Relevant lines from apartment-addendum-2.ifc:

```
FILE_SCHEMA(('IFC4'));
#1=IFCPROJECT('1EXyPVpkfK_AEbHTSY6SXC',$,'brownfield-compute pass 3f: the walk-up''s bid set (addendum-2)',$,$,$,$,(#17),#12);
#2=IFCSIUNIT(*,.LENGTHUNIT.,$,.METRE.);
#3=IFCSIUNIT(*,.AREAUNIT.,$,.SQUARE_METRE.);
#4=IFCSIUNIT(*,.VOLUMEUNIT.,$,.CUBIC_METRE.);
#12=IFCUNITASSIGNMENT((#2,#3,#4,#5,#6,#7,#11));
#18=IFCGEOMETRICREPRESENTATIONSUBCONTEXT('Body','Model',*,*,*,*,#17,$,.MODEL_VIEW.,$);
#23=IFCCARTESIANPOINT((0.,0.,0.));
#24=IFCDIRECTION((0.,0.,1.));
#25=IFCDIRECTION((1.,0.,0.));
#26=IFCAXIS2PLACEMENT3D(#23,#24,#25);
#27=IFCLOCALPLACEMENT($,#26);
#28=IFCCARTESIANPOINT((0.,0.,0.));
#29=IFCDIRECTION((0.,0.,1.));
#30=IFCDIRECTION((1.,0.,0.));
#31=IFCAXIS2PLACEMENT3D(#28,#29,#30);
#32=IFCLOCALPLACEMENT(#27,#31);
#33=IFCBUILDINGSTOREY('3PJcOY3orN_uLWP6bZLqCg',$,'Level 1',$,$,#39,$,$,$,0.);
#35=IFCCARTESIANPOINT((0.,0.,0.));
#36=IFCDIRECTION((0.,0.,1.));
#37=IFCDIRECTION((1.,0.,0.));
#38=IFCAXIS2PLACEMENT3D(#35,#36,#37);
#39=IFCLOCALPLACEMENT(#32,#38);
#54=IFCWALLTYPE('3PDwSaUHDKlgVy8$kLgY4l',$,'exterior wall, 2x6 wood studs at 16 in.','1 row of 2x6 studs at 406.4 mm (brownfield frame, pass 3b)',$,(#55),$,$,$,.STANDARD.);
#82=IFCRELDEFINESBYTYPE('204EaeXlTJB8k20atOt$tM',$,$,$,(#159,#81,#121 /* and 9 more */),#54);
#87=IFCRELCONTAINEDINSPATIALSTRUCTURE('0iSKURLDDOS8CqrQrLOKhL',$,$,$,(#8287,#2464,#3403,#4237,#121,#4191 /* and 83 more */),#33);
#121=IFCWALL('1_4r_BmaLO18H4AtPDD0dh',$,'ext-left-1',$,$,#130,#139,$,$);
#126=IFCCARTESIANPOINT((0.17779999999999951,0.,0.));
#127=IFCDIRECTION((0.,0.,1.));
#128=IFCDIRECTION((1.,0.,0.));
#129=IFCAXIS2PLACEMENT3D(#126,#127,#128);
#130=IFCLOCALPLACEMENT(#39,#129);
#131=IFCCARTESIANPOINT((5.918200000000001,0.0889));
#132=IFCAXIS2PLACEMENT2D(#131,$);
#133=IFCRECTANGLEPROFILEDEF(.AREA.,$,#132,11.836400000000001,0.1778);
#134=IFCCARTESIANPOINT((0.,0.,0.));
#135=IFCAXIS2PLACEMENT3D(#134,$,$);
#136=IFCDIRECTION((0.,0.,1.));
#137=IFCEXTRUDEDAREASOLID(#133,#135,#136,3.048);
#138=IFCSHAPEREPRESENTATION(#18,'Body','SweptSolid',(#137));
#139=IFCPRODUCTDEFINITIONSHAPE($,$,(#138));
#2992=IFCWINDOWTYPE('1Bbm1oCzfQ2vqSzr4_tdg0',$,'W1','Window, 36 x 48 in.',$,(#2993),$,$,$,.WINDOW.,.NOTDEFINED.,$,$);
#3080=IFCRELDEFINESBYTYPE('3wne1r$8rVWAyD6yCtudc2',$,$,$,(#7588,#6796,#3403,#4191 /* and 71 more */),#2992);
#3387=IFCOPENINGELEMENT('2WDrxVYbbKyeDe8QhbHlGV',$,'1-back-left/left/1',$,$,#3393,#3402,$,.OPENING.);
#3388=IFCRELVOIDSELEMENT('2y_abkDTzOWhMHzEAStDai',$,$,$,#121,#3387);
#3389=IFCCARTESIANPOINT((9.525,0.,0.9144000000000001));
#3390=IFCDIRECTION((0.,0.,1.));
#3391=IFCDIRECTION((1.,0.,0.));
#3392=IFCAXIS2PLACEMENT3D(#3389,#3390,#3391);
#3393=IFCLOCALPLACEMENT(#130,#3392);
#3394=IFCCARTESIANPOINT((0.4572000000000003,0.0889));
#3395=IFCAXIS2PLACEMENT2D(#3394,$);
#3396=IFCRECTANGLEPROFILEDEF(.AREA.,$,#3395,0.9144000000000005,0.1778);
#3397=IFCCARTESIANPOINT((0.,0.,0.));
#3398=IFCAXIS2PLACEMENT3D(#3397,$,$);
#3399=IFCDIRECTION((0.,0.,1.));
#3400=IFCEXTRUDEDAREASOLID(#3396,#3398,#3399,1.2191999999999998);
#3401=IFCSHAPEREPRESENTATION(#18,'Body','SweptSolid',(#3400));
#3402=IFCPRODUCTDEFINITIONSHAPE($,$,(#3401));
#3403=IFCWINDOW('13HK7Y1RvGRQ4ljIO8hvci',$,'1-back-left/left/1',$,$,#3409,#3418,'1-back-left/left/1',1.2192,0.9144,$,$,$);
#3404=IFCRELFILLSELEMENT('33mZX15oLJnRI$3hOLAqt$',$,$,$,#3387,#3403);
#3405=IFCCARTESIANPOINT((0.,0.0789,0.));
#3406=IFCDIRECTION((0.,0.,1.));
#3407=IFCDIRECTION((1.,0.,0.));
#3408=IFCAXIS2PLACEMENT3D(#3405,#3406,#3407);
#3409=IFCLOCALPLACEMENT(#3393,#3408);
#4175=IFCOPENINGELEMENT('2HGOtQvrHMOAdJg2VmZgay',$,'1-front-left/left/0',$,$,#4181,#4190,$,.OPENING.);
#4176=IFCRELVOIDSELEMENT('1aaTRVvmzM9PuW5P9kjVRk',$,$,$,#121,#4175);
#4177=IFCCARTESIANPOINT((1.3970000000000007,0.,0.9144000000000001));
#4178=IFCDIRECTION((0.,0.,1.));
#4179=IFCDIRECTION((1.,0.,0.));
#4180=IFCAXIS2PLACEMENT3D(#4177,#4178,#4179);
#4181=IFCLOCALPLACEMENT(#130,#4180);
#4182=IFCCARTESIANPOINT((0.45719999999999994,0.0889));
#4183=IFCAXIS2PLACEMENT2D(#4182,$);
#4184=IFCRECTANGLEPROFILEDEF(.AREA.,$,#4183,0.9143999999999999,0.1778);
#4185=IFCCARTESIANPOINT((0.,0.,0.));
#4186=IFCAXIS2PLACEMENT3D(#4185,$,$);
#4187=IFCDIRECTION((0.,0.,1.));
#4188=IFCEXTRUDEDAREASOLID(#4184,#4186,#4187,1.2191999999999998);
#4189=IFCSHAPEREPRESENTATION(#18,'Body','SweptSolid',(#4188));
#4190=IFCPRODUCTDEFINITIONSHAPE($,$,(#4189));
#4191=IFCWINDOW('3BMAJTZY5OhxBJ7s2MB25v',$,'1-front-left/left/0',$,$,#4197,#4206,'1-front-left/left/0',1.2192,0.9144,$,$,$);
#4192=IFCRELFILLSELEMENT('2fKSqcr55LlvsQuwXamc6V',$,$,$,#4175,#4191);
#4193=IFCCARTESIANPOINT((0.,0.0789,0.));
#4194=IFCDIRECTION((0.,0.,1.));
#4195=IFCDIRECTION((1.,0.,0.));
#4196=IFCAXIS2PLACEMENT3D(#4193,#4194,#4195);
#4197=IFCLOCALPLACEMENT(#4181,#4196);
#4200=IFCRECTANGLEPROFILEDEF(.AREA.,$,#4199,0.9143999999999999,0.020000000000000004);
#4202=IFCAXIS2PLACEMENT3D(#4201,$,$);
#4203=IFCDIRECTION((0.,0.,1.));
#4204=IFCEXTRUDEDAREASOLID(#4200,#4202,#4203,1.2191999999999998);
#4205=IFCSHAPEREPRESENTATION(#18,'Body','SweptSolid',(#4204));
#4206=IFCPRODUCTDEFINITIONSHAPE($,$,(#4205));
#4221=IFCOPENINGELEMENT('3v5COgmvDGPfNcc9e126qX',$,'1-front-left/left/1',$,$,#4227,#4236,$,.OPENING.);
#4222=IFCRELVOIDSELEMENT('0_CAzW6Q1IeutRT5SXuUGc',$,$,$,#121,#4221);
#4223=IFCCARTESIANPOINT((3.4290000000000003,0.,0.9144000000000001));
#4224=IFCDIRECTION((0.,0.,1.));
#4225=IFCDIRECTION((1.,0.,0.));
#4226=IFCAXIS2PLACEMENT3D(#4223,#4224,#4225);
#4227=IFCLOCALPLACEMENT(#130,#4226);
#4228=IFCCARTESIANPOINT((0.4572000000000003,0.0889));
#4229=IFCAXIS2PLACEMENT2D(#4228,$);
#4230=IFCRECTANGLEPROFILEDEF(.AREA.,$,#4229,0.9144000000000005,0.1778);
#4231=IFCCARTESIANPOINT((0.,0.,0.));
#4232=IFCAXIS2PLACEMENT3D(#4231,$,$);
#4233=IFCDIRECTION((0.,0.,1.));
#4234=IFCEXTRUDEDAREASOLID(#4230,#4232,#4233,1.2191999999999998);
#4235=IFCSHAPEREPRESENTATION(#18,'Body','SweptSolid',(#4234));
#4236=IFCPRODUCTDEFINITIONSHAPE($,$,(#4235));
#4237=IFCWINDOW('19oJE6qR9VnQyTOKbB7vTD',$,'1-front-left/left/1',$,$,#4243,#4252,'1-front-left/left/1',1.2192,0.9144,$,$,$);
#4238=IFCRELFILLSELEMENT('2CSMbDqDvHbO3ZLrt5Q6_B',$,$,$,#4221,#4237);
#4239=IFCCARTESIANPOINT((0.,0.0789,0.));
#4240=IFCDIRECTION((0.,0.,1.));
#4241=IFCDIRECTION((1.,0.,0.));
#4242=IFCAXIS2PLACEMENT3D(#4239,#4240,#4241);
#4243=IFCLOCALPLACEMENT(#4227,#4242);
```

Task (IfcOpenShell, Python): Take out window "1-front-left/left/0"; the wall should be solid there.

```python
import ifcopenshell
import ifcopenshell.api.feature
import ifcopenshell.api.root
import ifcopenshell.geom
import ifcopenshell.util.shape

model = ifcopenshell.open("apartment-addendum-2.ifc")
settings = ifcopenshell.geom.settings()


def volume(element):
    """Net volume in cubic metres, openings subtracted."""
    shape = ifcopenshell.geom.create_shape(settings, element)
    return ifcopenshell.util.shape.get_volume(shape.geometry)


window = model.by_guid("3BMAJTZY5OhxBJ7s2MB25v")
opening = window.FillsVoids[0].RelatingOpeningElement
wall = opening.VoidsElements[0].RelatingBuildingElement
before = volume(wall)

ifcopenshell.api.root.remove_product(model, product=window)
ifcopenshell.api.feature.remove_feature(model, feature=opening)

after = volume(wall)

print(f"wall volume {before:.3f} -> {after:.3f} m3")

model.write("apartment-addendum-2_rev.ifc")
```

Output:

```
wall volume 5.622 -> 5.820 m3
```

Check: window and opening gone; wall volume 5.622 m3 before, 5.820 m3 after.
